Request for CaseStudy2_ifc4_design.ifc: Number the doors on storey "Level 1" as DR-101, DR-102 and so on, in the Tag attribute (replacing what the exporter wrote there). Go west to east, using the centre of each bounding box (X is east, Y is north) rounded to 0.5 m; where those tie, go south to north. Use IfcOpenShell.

First a look at what the model holds.

```python
import ifcopenshell
import ifcopenshell.util.element
import ifcopenshell.util.placement

model = ifcopenshell.open("CaseStudy2_ifc4_design.ifc")
print(model.schema)
storey = next(s for s in model.by_type("IfcBuildingStorey") if s.Name == "Level 1")
doors = [e for e in ifcopenshell.util.element.get_decomposition(storey) if e.is_a("IfcDoor")]
for e in sorted(doors, key=lambda e: e.id()):
    origin = ifcopenshell.util.placement.get_local_placement(e.ObjectPlacement)[:3, 3]
    print(e.id(), e.Tag, e.Name, origin.round(2) + 0.0, sep=" | ")
```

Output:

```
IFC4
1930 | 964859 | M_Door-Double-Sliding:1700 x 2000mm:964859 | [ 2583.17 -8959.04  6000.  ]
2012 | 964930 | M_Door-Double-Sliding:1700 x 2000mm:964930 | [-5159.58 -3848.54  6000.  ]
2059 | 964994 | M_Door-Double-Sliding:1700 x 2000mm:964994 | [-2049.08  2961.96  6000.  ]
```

```python
import ifcopenshell
import ifcopenshell.geom
import ifcopenshell.util.element
import ifcopenshell.util.shape

model = ifcopenshell.open("CaseStudy2_ifc4_design.ifc")
settings = ifcopenshell.geom.settings()
settings.set("use-world-coords", True)


def centre(element):
    shape = ifcopenshell.geom.create_shape(settings, element)
    return ifcopenshell.util.shape.get_bbox_centroid(shape.geometry)


storey = next(s for s in model.by_type("IfcBuildingStorey") if s.Name == "Level 1")
doors = [e for e in ifcopenshell.util.element.get_decomposition(storey) if e.is_a("IfcDoor")]

# Insertion points can sit at a corner or the storey origin, so sort by the geometry (in metres).
centres = {e: centre(e) for e in doors}
doors.sort(key=lambda e: (round(centres[e][0] / 0.5), centres[e][1]))

for i, e in enumerate(doors, start=1):
    number = f"DR-1{i:02d}"
    e.Tag = number
    print(e.id(), number)

model.write("CaseStudy2_ifc4_design_edited.ifc")
```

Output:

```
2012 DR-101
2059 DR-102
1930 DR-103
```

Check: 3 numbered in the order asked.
